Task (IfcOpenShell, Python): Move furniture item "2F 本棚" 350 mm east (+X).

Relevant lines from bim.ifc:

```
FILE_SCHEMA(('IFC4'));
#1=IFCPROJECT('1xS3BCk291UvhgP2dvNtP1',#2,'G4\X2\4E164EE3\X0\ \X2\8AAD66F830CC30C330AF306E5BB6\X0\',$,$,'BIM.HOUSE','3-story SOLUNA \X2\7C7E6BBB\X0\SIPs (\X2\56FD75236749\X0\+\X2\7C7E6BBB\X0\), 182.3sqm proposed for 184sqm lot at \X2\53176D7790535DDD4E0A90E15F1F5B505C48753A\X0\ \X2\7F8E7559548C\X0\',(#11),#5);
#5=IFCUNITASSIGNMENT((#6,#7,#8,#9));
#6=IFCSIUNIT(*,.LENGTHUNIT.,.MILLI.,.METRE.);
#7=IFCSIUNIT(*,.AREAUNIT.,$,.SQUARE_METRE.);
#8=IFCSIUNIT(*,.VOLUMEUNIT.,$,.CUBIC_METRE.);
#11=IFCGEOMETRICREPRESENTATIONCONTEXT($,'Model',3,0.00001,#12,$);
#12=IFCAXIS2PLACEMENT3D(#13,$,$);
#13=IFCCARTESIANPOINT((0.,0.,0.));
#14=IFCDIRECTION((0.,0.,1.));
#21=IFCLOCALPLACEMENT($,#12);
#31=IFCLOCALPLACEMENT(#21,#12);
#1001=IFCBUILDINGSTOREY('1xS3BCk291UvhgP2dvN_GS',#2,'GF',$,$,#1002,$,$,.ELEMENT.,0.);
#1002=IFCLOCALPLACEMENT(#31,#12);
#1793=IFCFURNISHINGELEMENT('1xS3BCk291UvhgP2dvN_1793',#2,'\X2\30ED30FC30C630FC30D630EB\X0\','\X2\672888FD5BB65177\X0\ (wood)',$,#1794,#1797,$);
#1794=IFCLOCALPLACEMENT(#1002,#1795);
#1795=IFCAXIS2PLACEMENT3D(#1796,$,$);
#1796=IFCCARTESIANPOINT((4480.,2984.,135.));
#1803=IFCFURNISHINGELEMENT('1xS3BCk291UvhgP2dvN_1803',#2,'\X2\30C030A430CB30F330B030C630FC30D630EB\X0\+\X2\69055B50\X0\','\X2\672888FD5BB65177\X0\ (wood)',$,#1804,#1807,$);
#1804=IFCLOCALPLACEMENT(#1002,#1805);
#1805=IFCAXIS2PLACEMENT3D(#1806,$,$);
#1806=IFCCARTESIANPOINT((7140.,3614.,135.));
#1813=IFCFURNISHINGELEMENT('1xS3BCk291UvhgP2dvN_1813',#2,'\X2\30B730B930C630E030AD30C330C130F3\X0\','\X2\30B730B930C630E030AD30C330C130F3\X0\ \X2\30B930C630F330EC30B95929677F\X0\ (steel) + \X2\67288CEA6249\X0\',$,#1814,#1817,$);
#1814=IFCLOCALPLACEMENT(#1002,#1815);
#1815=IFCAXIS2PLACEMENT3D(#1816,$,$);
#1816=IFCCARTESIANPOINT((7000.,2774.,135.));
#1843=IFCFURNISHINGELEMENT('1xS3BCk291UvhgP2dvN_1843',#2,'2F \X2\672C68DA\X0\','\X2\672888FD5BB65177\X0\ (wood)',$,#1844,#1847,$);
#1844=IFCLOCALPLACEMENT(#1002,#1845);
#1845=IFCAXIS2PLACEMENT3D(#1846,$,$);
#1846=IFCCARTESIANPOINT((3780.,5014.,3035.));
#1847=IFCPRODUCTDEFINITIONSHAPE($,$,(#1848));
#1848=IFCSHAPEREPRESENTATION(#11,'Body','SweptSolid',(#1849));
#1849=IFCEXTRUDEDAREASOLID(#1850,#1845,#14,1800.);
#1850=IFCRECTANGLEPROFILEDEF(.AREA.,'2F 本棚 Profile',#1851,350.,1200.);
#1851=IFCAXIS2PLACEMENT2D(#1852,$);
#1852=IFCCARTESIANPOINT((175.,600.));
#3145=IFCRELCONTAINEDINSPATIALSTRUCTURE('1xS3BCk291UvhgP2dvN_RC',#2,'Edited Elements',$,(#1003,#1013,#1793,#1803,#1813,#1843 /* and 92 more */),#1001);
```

```python
import ifcopenshell
import ifcopenshell.api.geometry
import ifcopenshell.util.placement
import ifcopenshell.util.unit

model = ifcopenshell.open("bim.ifc")
unit_scale = ifcopenshell.util.unit.calculate_unit_scale(model)

item = model.by_guid("1xS3BCk291UvhgP2dvN_1843")
matrix = ifcopenshell.util.placement.get_local_placement(item.ObjectPlacement)
matrix[0, 3] += 0.35 / unit_scale
ifcopenshell.api.geometry.edit_object_placement(model, product=item, matrix=matrix, is_si=False)

print(ifcopenshell.util.placement.get_local_placement(item.ObjectPlacement).round(3) + 0.0)

model.write("bim_edited.ifc")
```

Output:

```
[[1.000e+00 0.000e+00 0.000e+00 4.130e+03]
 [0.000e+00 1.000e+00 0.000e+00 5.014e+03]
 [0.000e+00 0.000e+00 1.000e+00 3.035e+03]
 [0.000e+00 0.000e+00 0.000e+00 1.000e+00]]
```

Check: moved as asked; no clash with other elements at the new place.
